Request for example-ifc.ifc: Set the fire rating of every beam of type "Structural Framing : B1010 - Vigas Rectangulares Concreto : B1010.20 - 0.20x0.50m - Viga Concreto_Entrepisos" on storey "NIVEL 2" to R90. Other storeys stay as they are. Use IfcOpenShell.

First a look at what the model holds.

```python
import ifcopenshell
import ifcopenshell.util.element

model = ifcopenshell.open("example-ifc.ifc")
print(model.schema)
storey = next(s for s in model.by_type("IfcBuildingStorey") if s.Name == "NIVEL 2")
beams = [e for e in ifcopenshell.util.element.get_decomposition(storey) if e.is_a("IfcBeam")]
seen = {}
for e in beams:
    element_type = ifcopenshell.util.element.get_type(e)
    key = (element_type.Name if element_type != e and element_type else None, ifcopenshell.util.element.get_pset(e, "Pset_BeamCommon", "FireRating"))
    seen[key] = seen.get(key, 0) + 1
for (name, value), count in sorted(seen.items(), key=str):
    print(count, "x", name, "|", value)
```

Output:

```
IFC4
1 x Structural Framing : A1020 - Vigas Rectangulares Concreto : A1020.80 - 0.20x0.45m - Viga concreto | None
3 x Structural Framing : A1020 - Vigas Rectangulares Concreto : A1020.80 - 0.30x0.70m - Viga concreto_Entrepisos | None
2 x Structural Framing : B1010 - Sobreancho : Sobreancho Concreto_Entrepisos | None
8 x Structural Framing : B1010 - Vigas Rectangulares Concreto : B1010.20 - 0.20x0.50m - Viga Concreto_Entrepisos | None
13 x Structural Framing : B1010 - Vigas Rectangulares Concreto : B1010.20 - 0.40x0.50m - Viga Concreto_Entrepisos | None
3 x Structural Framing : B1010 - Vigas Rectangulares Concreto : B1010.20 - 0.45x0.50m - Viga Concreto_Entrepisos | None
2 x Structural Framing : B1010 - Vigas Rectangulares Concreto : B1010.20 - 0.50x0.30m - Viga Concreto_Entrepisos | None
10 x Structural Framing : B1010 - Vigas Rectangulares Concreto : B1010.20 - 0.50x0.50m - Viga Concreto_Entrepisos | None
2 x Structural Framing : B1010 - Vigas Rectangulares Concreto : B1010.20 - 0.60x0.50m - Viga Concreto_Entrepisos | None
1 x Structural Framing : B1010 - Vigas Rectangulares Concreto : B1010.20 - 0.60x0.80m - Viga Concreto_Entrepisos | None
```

```python
import ifcopenshell
import ifcopenshell.api.pset
import ifcopenshell.util.element

model = ifcopenshell.open("example-ifc.ifc")

storey = next(s for s in model.by_type("IfcBuildingStorey") if s.Name == "NIVEL 2")
beams = [e for e in ifcopenshell.util.element.get_decomposition(storey) if e.is_a("IfcBeam")]

count = 0
for e in beams:
    element_type = ifcopenshell.util.element.get_type(e)
    if element_type in (None, e) or element_type.Name != "Structural Framing : B1010 - Vigas Rectangulares Concreto : B1010.20 - 0.20x0.50m - Viga Concreto_Entrepisos":
        continue
    # add_pset returns the element's existing set when there is one.
    pset = ifcopenshell.api.pset.add_pset(model, product=e, name="Pset_BeamCommon")
    ifcopenshell.api.pset.edit_pset(model, pset=pset, properties={"FireRating": "R90"})
    count += 1

print(count, "beams updated")

model.write("example-ifc-out.ifc")
```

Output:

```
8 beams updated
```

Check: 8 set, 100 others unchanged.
